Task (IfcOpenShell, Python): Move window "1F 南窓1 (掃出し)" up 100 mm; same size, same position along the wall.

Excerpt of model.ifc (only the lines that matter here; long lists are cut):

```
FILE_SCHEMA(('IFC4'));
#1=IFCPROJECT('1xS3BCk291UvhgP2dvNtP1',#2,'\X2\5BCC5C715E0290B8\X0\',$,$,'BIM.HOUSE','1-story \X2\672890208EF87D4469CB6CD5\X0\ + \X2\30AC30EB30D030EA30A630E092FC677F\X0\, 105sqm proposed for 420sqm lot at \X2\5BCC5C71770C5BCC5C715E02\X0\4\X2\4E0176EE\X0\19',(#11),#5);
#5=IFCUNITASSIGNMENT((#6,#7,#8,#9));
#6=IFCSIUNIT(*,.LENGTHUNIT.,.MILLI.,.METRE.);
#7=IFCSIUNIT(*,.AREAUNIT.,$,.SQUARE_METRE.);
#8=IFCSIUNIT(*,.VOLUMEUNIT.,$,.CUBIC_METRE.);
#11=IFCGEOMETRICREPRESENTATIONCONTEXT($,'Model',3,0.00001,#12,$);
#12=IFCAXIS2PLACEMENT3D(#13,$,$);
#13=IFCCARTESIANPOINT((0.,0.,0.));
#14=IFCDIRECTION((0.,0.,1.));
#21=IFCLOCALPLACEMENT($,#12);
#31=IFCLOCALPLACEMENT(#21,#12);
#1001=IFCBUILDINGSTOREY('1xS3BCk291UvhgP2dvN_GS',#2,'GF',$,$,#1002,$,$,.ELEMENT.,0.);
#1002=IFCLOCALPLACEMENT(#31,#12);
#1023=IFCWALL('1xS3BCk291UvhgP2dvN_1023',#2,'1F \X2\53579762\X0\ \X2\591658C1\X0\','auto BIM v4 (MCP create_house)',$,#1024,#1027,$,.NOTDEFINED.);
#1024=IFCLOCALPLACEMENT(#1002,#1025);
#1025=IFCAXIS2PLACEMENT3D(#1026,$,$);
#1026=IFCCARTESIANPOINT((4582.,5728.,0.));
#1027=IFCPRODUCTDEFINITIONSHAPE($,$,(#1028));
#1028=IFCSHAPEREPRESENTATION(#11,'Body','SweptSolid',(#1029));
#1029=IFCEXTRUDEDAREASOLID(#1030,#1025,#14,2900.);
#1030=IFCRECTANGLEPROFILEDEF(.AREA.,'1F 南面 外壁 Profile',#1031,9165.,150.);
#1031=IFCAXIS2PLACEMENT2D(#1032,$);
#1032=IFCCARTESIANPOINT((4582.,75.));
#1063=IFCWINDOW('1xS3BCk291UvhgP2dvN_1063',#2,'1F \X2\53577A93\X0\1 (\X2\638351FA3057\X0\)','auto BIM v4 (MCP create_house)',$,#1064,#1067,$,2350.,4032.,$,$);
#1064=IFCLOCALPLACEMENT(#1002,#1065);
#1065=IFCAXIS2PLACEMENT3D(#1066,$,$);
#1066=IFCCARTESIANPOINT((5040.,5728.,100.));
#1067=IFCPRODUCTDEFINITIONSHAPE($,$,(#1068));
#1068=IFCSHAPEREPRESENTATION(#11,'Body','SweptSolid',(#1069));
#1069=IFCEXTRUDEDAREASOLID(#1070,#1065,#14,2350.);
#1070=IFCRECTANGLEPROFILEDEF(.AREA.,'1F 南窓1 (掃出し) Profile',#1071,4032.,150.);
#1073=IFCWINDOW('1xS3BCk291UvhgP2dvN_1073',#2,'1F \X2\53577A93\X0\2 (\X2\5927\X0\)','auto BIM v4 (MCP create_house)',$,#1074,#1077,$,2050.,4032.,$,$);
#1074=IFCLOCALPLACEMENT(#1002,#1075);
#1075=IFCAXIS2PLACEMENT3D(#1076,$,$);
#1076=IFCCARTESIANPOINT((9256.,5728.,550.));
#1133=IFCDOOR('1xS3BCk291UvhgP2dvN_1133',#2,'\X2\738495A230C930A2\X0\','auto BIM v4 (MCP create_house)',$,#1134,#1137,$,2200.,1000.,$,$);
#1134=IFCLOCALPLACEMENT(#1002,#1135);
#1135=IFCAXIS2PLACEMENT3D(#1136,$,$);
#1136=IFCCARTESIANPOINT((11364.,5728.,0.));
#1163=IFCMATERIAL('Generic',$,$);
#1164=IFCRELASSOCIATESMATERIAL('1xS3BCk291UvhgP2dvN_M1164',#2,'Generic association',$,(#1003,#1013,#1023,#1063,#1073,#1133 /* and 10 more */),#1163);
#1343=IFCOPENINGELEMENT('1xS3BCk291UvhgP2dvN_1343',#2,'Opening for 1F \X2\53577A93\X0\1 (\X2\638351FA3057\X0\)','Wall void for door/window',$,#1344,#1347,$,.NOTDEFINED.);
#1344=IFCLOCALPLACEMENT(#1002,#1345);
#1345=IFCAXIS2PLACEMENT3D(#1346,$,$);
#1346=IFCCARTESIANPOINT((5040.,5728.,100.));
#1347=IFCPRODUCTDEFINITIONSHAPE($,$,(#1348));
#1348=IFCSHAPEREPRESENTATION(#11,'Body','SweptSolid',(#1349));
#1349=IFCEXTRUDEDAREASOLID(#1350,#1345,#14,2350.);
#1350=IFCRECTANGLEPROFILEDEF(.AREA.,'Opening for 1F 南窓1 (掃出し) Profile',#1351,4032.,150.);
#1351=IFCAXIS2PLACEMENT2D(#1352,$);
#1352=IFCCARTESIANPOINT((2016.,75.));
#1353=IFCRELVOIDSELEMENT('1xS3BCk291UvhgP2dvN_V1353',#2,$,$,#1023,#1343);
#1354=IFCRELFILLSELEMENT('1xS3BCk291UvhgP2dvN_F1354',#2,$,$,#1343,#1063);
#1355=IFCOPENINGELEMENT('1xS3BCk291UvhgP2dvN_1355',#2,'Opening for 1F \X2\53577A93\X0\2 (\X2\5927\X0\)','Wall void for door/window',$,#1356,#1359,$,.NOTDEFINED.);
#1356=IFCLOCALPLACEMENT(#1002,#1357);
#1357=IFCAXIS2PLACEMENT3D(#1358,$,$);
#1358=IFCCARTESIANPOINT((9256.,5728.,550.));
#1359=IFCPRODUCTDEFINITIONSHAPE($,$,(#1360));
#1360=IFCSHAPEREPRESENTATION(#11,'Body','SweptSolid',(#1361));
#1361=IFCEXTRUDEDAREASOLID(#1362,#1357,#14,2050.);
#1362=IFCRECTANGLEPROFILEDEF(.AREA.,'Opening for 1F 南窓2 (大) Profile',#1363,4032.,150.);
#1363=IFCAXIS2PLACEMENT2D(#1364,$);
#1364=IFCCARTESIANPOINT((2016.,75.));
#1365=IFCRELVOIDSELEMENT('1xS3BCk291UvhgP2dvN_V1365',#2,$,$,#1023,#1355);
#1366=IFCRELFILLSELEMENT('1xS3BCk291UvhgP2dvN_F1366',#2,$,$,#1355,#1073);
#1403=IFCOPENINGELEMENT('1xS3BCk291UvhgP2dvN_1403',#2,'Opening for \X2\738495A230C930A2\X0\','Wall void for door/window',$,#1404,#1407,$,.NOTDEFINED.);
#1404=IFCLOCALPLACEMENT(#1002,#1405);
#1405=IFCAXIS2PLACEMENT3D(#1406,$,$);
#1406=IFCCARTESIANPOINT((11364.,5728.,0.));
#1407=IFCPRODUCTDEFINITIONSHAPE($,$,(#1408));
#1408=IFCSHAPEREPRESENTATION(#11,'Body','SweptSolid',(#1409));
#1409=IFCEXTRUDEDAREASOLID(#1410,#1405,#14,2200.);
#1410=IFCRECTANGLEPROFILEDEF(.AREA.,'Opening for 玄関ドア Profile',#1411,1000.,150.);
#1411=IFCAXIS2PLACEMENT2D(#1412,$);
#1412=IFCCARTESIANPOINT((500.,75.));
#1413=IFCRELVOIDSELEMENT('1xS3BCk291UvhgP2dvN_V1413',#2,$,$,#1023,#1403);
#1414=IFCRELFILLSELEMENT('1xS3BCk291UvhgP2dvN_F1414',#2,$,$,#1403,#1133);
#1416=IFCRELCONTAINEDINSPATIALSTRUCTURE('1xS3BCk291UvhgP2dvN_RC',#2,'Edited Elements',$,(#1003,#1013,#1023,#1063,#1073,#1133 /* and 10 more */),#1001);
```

```python
import numpy as np
import ifcopenshell
import ifcopenshell.api.geometry
import ifcopenshell.util.placement
import ifcopenshell.util.unit

model = ifcopenshell.open("model.ifc")
unit_scale = ifcopenshell.util.unit.calculate_unit_scale(model)

window = model.by_guid("1xS3BCk291UvhgP2dvN_1063")
opening = window.FillsVoids[0].RelatingOpeningElement
dz = 0.1 / unit_scale

shift = np.array([0.0, 0.0, dz])
# The window is not placed relative to its opening, so move both.
for product in (opening, window):
    matrix = ifcopenshell.util.placement.get_local_placement(product.ObjectPlacement)
    matrix[:3, 3] += shift
    ifcopenshell.api.geometry.edit_object_placement(model, product=product, matrix=matrix, is_si=False)

print(f"moved by {dz * unit_scale:+.3f} m")

model.write("model_rev.ifc")
```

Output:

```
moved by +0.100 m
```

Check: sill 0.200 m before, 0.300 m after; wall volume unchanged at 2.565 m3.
